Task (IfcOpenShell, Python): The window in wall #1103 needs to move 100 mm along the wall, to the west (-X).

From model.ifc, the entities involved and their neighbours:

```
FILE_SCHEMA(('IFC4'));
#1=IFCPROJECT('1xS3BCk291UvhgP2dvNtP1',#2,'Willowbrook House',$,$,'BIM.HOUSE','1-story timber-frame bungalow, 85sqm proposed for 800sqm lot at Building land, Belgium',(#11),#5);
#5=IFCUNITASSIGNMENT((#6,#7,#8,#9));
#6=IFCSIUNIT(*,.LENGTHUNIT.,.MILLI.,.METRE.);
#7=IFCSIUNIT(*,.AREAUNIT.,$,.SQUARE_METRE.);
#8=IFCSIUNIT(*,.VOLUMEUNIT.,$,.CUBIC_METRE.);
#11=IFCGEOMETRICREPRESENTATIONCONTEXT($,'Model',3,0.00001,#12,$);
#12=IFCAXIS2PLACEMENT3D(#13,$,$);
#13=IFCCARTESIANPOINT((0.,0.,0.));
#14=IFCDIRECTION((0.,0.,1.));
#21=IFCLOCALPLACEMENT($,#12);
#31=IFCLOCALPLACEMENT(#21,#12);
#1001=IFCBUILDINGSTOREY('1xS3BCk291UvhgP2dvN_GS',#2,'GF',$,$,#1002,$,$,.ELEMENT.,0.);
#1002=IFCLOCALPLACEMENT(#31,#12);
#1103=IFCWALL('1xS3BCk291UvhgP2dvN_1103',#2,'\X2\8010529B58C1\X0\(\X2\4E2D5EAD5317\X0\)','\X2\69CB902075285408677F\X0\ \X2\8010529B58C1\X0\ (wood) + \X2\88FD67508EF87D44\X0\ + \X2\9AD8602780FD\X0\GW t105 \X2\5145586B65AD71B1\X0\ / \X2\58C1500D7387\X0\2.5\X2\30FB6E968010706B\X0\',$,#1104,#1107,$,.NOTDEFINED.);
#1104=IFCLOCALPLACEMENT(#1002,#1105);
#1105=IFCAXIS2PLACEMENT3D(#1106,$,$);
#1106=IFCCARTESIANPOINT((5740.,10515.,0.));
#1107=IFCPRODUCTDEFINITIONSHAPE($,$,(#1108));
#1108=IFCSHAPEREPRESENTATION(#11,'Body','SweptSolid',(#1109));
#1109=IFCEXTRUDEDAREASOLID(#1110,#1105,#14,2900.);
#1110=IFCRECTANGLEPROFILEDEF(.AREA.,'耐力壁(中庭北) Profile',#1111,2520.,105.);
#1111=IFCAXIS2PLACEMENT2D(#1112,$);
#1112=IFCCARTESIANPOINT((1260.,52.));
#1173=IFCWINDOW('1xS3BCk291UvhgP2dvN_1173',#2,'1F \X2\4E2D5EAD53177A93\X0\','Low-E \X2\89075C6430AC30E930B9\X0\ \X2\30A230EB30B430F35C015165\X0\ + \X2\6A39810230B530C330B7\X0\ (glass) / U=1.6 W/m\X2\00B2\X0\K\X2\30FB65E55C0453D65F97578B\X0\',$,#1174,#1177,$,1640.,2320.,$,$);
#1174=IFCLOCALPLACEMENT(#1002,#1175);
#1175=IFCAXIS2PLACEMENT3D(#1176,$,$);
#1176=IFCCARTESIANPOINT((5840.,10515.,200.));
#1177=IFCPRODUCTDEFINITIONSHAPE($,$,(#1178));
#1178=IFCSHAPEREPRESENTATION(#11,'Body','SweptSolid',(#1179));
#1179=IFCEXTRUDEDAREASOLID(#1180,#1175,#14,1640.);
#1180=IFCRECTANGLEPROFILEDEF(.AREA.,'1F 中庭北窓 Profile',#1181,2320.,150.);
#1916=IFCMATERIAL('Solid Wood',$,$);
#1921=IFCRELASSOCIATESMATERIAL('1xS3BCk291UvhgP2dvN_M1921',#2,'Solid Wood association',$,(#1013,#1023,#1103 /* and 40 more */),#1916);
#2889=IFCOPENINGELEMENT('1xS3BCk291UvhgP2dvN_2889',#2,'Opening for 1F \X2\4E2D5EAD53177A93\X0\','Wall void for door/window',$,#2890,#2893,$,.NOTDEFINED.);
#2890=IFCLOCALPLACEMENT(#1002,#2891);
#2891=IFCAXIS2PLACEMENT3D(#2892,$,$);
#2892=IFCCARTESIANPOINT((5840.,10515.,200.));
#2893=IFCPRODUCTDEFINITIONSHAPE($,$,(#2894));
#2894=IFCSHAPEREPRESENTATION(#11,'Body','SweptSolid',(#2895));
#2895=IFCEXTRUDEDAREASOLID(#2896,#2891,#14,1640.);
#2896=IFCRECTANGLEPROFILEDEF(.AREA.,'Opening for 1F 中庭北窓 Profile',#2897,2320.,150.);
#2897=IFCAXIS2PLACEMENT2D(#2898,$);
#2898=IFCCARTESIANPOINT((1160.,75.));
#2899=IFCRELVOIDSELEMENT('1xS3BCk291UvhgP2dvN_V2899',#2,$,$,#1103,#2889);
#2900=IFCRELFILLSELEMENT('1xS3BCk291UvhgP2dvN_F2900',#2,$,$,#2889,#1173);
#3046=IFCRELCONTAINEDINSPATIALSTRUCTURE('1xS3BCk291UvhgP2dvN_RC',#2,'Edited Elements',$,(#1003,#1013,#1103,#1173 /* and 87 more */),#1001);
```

```python
import ifcopenshell
import ifcopenshell.api.geometry
import ifcopenshell.util.placement
import ifcopenshell.util.unit

model = ifcopenshell.open("model.ifc")
unit_scale = ifcopenshell.util.unit.calculate_unit_scale(model)

window = model.by_guid("1xS3BCk291UvhgP2dvN_1173")
opening = window.FillsVoids[0].RelatingOpeningElement
wall = opening.VoidsElements[0].RelatingBuildingElement

wall_matrix = ifcopenshell.util.placement.get_local_placement(wall.ObjectPlacement)
shift = wall_matrix[:3, 0] * -0.1 / unit_scale
before = ifcopenshell.util.placement.get_local_placement(window.ObjectPlacement)[:3, 3].copy()

# The window is not placed relative to its opening, so move both.
for product in (opening, window):
    matrix = ifcopenshell.util.placement.get_local_placement(product.ObjectPlacement)
    matrix[:3, 3] += shift
    ifcopenshell.api.geometry.edit_object_placement(model, product=product, matrix=matrix, is_si=False)

after = ifcopenshell.util.placement.get_local_placement(window.ObjectPlacement)[:3, 3]
print("window moved by", (after - before).round(3) + 0.0)

model.write("model_updated.ifc")
```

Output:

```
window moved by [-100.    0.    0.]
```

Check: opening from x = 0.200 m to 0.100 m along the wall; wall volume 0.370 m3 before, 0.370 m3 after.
